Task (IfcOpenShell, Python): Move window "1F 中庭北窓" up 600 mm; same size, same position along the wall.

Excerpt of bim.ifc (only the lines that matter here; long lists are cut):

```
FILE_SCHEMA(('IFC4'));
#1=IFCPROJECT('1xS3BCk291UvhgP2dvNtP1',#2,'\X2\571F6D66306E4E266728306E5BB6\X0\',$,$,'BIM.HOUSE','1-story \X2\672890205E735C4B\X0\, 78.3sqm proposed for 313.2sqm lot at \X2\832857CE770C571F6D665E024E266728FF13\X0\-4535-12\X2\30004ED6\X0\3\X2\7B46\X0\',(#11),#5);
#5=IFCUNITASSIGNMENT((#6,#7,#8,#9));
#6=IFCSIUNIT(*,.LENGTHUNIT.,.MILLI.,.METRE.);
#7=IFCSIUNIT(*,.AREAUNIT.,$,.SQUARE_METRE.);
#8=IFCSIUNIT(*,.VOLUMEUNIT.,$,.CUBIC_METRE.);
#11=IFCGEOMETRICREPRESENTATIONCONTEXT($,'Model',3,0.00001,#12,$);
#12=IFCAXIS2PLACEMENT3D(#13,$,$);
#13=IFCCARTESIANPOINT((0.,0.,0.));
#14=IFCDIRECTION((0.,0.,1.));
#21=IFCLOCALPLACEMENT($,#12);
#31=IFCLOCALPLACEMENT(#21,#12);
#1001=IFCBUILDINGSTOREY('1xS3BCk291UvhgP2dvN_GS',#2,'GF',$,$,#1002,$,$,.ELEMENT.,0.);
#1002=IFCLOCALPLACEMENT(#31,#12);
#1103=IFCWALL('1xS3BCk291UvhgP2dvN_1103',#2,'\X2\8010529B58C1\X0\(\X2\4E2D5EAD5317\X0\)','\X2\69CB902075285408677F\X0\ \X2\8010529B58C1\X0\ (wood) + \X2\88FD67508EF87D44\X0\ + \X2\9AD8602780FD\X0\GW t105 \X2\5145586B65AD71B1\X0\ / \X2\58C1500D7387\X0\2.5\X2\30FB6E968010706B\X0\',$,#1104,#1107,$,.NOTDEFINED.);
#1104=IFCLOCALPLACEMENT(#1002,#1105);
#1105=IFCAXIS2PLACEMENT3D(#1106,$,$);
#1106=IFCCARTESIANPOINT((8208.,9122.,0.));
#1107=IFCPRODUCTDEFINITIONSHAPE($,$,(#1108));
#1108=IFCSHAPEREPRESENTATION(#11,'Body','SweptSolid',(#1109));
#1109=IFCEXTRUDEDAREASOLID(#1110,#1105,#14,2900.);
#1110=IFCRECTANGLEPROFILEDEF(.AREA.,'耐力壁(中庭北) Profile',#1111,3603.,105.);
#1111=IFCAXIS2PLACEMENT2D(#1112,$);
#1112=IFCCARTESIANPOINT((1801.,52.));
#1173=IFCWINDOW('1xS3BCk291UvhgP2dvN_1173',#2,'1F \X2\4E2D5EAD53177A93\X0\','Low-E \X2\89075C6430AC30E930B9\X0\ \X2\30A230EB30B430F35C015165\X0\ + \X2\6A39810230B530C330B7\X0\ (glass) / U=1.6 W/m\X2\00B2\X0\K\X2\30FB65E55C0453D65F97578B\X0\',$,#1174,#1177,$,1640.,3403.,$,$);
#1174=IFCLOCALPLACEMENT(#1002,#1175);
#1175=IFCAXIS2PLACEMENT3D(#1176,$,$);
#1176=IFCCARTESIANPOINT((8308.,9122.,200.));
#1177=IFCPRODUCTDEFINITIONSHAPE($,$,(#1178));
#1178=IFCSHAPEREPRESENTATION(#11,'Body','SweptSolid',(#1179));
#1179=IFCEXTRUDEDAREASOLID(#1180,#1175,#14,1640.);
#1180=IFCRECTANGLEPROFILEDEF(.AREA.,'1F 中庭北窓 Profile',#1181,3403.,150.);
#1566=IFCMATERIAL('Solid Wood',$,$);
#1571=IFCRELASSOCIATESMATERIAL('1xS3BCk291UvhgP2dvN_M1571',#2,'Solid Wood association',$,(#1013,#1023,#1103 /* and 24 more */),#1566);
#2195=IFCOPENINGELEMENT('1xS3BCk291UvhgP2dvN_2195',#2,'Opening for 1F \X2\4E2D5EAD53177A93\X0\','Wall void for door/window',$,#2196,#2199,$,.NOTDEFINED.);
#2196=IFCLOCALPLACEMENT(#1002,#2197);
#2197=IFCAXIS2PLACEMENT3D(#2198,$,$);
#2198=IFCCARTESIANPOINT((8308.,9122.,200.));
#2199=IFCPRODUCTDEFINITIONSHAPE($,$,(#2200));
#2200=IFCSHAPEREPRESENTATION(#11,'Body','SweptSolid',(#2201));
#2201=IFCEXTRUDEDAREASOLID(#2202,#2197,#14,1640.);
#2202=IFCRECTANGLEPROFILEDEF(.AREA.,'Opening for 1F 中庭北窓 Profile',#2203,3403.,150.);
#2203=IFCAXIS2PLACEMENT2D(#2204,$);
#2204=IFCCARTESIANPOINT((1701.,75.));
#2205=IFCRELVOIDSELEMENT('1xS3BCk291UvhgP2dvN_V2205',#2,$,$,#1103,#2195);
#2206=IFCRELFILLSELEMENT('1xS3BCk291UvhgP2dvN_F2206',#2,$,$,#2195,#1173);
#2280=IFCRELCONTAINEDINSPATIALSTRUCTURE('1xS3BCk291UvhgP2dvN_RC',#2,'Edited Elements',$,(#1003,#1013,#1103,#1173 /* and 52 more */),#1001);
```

```python
import numpy as np
import ifcopenshell
import ifcopenshell.api.geometry
import ifcopenshell.util.placement
import ifcopenshell.util.unit

model = ifcopenshell.open("bim.ifc")
unit_scale = ifcopenshell.util.unit.calculate_unit_scale(model)

window = model.by_id(1173)
opening = window.FillsVoids[0].RelatingOpeningElement
dz = 0.6 / unit_scale

shift = np.array([0.0, 0.0, dz])
# The window is not placed relative to its opening, so move both.
for product in (opening, window):
    matrix = ifcopenshell.util.placement.get_local_placement(product.ObjectPlacement)
    matrix[:3, 3] += shift
    ifcopenshell.api.geometry.edit_object_placement(model, product=product, matrix=matrix, is_si=False)

print(f"moved by {dz * unit_scale:+.3f} m")

model.write("bim-out.ifc")
```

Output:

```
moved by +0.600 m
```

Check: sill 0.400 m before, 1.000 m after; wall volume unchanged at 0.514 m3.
